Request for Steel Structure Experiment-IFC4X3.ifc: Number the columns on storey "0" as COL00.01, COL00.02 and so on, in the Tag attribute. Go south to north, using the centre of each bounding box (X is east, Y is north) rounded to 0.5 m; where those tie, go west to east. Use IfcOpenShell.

First a look at what the model holds.

```python
import ifcopenshell
import ifcopenshell.util.element
import ifcopenshell.util.placement

model = ifcopenshell.open("Steel Structure Experiment-IFC4X3.ifc")
print(model.schema)
storey = next(s for s in model.by_type("IfcBuildingStorey") if s.Name == "0")
columns = [e for e in ifcopenshell.util.element.get_decomposition(storey) if e.is_a("IfcColumn")]
for e in sorted(columns, key=lambda e: e.id()):
    origin = ifcopenshell.util.placement.get_local_placement(e.ObjectPlacement)[:3, 3]
    print(e.id(), e.Tag, e.Name, origin.round(2) + 0.0, sep=" | ")
```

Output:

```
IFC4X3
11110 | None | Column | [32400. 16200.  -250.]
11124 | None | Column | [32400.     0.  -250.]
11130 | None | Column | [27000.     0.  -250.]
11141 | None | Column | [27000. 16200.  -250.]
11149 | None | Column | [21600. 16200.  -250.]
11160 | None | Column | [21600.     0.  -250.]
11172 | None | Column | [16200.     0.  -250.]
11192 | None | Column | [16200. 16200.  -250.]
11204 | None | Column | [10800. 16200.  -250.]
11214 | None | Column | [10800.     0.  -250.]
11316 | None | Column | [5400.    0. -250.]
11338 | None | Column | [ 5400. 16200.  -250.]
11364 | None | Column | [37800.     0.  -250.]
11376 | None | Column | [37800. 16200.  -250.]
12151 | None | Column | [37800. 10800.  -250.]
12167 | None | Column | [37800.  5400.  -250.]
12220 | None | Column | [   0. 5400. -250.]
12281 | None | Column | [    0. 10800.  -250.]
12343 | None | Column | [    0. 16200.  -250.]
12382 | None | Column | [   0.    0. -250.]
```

```python
import ifcopenshell
import ifcopenshell.geom
import ifcopenshell.util.element
import ifcopenshell.util.shape

model = ifcopenshell.open("Steel Structure Experiment-IFC4X3.ifc")
settings = ifcopenshell.geom.settings()
settings.set("use-world-coords", True)


def centre(element):
    shape = ifcopenshell.geom.create_shape(settings, element)
    return ifcopenshell.util.shape.get_bbox_centroid(shape.geometry)


storey = next(s for s in model.by_type("IfcBuildingStorey") if s.Name == "0")
columns = [e for e in ifcopenshell.util.element.get_decomposition(storey) if e.is_a("IfcColumn")]

# Insertion points can sit at a corner or the storey origin, so sort by the geometry (in metres).
centres = {e: centre(e) for e in columns}
columns.sort(key=lambda e: (round(centres[e][1] / 0.5), centres[e][0]))

for i, e in enumerate(columns, start=1):
    number = f"COL00.{i:02d}"
    e.Tag = number
    print(e.id(), number)

model.write("Steel Structure Experiment-IFC4X3_rev.ifc")
```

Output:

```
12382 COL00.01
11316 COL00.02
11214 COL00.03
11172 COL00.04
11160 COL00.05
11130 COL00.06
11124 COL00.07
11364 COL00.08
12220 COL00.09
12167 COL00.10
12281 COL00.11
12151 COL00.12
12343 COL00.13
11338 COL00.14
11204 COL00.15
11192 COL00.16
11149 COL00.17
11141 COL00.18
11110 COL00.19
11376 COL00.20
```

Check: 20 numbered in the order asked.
